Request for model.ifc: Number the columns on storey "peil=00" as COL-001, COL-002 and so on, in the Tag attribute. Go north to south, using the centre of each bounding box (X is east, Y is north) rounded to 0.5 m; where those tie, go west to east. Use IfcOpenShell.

First a look at what the model holds.

```python
import ifcopenshell
import ifcopenshell.util.element
import ifcopenshell.util.placement

model = ifcopenshell.open("model.ifc")
print(model.schema)
storey = next(s for s in model.by_type("IfcBuildingStorey") if s.Name == "peil=00")
columns = [e for e in ifcopenshell.util.element.get_decomposition(storey) if e.is_a("IfcColumn")]
for e in sorted(columns, key=lambda e: e.id()):
    origin = ifcopenshell.util.placement.get_local_placement(e.ObjectPlacement)[:3, 3]
    print(e.id(), e.Tag, e.Name, origin.round(2) + 0.0, sep=" | ")
```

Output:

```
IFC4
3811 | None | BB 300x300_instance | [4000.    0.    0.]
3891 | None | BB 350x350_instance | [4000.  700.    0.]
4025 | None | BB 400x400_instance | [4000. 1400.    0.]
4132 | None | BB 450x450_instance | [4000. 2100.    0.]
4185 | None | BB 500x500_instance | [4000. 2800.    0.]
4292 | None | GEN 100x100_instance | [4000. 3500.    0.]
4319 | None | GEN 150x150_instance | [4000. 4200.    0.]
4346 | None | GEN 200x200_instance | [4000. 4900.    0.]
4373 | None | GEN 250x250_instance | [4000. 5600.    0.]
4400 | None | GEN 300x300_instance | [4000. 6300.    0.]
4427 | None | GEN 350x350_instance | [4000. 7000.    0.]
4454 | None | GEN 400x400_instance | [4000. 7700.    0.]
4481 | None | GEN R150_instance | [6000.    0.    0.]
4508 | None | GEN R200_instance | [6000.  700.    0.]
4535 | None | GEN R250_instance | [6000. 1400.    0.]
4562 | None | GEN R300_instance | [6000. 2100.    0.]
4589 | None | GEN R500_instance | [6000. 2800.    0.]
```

```python
import ifcopenshell
import ifcopenshell.geom
import ifcopenshell.util.element
import ifcopenshell.util.shape

model = ifcopenshell.open("model.ifc")
settings = ifcopenshell.geom.settings()
settings.set("use-world-coords", True)


def centre(element):
    shape = ifcopenshell.geom.create_shape(settings, element)
    return ifcopenshell.util.shape.get_bbox_centroid(shape.geometry)


storey = next(s for s in model.by_type("IfcBuildingStorey") if s.Name == "peil=00")
columns = [e for e in ifcopenshell.util.element.get_decomposition(storey) if e.is_a("IfcColumn")]

# Insertion points can sit at a corner or the storey origin, so sort by the geometry (in metres).
centres = {e: centre(e) for e in columns}
columns.sort(key=lambda e: (-round(centres[e][1] / 0.5), centres[e][0]))

for i, e in enumerate(columns, start=1):
    number = f"COL-0{i:02d}"
    e.Tag = number
    print(e.id(), number)

model.write("model_v2.ifc")
```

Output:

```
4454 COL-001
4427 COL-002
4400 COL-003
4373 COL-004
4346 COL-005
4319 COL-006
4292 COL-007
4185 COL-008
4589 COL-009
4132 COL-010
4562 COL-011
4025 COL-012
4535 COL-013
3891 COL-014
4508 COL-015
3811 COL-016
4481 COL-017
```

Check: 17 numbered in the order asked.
